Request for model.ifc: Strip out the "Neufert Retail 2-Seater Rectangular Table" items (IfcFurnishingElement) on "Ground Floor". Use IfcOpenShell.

First a look at what the model holds.

```python
import ifcopenshell
import ifcopenshell.util.element

model = ifcopenshell.open("model.ifc")
print(model.schema)
storey = next(s for s in model.by_type("IfcBuildingStorey") if s.Name == "Ground Floor")
furniture = [e for e in ifcopenshell.util.element.get_decomposition(storey) if e.is_a("IfcFurnishingElement")]
seen = {}
for e in furniture:
    element_type = ifcopenshell.util.element.get_type(e)
    name = element_type.Name if element_type not in (None, e) else None
    seen[name] = seen.get(name, 0) + 1
for name, count in sorted(seen.items(), key=str):
    print(count, "x", name)
```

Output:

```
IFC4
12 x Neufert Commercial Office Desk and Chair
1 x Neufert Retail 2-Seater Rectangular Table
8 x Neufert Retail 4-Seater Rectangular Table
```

```python
import ifcopenshell
import ifcopenshell.api.root
import ifcopenshell.util.element

model = ifcopenshell.open("model.ifc")

storey = next(s for s in model.by_type("IfcBuildingStorey") if s.Name == "Ground Floor")
furniture = [e for e in ifcopenshell.util.element.get_decomposition(storey) if e.is_a("IfcFurnishingElement")]
targets = [e for e in furniture if (t := ifcopenshell.util.element.get_type(e)) not in (None, e) and t.Name == "Neufert Retail 2-Seater Rectangular Table"]

for e in targets:
    ifcopenshell.api.root.remove_product(model, product=e)
print(len(targets), "removed")

model.write("model-out.ifc")
```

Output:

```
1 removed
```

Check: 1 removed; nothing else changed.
